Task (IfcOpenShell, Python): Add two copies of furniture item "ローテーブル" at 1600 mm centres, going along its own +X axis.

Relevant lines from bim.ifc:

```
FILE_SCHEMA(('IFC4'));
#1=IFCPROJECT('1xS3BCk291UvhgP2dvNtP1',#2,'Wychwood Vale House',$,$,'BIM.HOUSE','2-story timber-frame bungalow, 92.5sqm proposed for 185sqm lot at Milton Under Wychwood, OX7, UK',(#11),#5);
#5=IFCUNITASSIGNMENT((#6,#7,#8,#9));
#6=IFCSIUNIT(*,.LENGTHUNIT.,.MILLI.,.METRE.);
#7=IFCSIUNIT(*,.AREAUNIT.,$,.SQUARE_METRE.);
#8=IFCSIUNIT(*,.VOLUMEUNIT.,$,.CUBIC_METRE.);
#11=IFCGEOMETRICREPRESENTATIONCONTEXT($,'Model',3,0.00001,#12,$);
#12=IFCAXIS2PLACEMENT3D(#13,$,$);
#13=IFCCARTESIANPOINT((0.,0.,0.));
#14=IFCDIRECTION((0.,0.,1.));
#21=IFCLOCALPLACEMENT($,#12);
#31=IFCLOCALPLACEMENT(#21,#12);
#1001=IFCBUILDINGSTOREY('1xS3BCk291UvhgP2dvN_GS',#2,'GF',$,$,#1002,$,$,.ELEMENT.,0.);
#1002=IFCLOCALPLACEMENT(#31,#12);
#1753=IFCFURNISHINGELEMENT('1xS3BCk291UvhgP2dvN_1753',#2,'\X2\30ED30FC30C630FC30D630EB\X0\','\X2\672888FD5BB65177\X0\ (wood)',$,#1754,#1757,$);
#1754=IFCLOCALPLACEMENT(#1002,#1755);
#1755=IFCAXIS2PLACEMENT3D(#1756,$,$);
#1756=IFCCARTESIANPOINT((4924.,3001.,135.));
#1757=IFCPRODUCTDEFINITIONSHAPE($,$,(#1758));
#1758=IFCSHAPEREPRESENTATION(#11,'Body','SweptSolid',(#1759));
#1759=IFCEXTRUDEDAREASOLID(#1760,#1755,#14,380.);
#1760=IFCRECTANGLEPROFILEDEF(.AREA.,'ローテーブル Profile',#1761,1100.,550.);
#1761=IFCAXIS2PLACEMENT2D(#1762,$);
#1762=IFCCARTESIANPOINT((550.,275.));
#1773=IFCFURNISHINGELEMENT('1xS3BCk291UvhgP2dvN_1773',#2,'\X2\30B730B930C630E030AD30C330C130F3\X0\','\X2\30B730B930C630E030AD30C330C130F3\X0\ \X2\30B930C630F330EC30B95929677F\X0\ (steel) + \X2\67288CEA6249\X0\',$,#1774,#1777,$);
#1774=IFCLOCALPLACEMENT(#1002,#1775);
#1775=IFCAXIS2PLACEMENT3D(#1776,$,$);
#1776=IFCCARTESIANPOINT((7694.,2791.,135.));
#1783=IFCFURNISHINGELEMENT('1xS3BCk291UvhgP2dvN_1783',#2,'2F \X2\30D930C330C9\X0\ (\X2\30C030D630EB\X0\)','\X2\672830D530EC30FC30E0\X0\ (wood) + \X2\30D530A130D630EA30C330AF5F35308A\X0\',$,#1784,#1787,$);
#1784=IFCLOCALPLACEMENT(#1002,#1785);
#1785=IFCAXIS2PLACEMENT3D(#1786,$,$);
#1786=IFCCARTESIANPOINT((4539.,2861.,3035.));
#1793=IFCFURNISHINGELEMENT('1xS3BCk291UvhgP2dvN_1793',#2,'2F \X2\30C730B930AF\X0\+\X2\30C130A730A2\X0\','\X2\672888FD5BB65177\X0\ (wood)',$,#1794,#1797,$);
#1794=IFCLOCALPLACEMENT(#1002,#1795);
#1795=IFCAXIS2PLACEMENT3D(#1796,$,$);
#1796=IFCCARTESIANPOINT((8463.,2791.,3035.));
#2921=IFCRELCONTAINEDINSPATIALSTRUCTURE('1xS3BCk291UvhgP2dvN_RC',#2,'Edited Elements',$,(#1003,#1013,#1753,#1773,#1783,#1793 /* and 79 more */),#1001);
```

```python
import ifcopenshell
import ifcopenshell.api.geometry
import ifcopenshell.api.root
import ifcopenshell.util.element
import ifcopenshell.util.placement
import ifcopenshell.util.unit

model = ifcopenshell.open("bim.ifc")
unit_scale = ifcopenshell.util.unit.calculate_unit_scale(model)


def reuse_history(source, copy):
    """copy_class also copies each property set's owner history, people and application; keep the originals."""
    for rel in copy.IsDefinedBy:
        if rel.is_a("IfcRelDefinesByProperties") and (history := rel.RelatingPropertyDefinition.OwnerHistory):
            rel.RelatingPropertyDefinition.OwnerHistory = source.OwnerHistory
            ifcopenshell.util.element.remove_deep2(model, history)


source = model.by_guid("1xS3BCk291UvhgP2dvN_1753")
base = ifcopenshell.util.placement.get_local_placement(source.ObjectPlacement)
step = base[:3, 0] * 1.6 / unit_scale

for i in range(1, 3):
    copy = ifcopenshell.api.root.copy_class(model, product=source)
    copy.Representation = ifcopenshell.util.element.copy_deep(
        model, source.Representation, exclude=["IfcGeometricRepresentationContext", "IfcRepresentationMap"]
    )
    reuse_history(source, copy)
    matrix = base.copy()
    matrix[:3, 3] += i * step
    print("added at", matrix[:3, 3].round(3) + 0.0)
    ifcopenshell.api.geometry.edit_object_placement(model, product=copy, matrix=matrix, is_si=False)

model.write("bim_edited.ifc")
```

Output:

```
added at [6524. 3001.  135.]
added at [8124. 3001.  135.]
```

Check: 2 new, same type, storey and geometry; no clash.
